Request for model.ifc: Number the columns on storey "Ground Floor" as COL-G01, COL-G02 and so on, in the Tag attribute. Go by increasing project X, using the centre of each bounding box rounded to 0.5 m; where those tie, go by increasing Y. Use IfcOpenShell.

First a look at what the model holds.

```python
import ifcopenshell
import ifcopenshell.util.element
import ifcopenshell.util.placement

model = ifcopenshell.open("model.ifc")
print(model.schema)
storey = next(s for s in model.by_type("IfcBuildingStorey") if s.Name == "Ground Floor")
columns = [e for e in ifcopenshell.util.element.get_decomposition(storey) if e.is_a("IfcColumn")]
for e in sorted(columns, key=lambda e: e.id()):
    origin = ifcopenshell.util.placement.get_local_placement(e.ObjectPlacement)[:3, 3]
    print(e.id(), e.Tag, e.Name, origin.round(2) + 0.0, sep=" | ")
```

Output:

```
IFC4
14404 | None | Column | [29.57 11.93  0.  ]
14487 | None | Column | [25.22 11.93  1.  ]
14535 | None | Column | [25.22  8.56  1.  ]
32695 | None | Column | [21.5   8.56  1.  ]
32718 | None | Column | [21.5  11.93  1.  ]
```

```python
import ifcopenshell
import ifcopenshell.geom
import ifcopenshell.util.element
import ifcopenshell.util.shape

model = ifcopenshell.open("model.ifc")
settings = ifcopenshell.geom.settings()
settings.set("use-world-coords", True)


def centre(element):
    shape = ifcopenshell.geom.create_shape(settings, element)
    return ifcopenshell.util.shape.get_bbox_centroid(shape.geometry)


storey = next(s for s in model.by_type("IfcBuildingStorey") if s.Name == "Ground Floor")
columns = [e for e in ifcopenshell.util.element.get_decomposition(storey) if e.is_a("IfcColumn")]

# Insertion points can sit at a corner or the storey origin, so sort by the geometry (in metres).
centres = {e: centre(e) for e in columns}
columns.sort(key=lambda e: (round(centres[e][0] / 0.5), centres[e][1]))

for i, e in enumerate(columns, start=1):
    number = f"COL-G{i:02d}"
    e.Tag = number
    print(e.id(), number)

model.write("model-out.ifc")
```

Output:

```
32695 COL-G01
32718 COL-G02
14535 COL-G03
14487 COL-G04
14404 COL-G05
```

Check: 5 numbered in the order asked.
